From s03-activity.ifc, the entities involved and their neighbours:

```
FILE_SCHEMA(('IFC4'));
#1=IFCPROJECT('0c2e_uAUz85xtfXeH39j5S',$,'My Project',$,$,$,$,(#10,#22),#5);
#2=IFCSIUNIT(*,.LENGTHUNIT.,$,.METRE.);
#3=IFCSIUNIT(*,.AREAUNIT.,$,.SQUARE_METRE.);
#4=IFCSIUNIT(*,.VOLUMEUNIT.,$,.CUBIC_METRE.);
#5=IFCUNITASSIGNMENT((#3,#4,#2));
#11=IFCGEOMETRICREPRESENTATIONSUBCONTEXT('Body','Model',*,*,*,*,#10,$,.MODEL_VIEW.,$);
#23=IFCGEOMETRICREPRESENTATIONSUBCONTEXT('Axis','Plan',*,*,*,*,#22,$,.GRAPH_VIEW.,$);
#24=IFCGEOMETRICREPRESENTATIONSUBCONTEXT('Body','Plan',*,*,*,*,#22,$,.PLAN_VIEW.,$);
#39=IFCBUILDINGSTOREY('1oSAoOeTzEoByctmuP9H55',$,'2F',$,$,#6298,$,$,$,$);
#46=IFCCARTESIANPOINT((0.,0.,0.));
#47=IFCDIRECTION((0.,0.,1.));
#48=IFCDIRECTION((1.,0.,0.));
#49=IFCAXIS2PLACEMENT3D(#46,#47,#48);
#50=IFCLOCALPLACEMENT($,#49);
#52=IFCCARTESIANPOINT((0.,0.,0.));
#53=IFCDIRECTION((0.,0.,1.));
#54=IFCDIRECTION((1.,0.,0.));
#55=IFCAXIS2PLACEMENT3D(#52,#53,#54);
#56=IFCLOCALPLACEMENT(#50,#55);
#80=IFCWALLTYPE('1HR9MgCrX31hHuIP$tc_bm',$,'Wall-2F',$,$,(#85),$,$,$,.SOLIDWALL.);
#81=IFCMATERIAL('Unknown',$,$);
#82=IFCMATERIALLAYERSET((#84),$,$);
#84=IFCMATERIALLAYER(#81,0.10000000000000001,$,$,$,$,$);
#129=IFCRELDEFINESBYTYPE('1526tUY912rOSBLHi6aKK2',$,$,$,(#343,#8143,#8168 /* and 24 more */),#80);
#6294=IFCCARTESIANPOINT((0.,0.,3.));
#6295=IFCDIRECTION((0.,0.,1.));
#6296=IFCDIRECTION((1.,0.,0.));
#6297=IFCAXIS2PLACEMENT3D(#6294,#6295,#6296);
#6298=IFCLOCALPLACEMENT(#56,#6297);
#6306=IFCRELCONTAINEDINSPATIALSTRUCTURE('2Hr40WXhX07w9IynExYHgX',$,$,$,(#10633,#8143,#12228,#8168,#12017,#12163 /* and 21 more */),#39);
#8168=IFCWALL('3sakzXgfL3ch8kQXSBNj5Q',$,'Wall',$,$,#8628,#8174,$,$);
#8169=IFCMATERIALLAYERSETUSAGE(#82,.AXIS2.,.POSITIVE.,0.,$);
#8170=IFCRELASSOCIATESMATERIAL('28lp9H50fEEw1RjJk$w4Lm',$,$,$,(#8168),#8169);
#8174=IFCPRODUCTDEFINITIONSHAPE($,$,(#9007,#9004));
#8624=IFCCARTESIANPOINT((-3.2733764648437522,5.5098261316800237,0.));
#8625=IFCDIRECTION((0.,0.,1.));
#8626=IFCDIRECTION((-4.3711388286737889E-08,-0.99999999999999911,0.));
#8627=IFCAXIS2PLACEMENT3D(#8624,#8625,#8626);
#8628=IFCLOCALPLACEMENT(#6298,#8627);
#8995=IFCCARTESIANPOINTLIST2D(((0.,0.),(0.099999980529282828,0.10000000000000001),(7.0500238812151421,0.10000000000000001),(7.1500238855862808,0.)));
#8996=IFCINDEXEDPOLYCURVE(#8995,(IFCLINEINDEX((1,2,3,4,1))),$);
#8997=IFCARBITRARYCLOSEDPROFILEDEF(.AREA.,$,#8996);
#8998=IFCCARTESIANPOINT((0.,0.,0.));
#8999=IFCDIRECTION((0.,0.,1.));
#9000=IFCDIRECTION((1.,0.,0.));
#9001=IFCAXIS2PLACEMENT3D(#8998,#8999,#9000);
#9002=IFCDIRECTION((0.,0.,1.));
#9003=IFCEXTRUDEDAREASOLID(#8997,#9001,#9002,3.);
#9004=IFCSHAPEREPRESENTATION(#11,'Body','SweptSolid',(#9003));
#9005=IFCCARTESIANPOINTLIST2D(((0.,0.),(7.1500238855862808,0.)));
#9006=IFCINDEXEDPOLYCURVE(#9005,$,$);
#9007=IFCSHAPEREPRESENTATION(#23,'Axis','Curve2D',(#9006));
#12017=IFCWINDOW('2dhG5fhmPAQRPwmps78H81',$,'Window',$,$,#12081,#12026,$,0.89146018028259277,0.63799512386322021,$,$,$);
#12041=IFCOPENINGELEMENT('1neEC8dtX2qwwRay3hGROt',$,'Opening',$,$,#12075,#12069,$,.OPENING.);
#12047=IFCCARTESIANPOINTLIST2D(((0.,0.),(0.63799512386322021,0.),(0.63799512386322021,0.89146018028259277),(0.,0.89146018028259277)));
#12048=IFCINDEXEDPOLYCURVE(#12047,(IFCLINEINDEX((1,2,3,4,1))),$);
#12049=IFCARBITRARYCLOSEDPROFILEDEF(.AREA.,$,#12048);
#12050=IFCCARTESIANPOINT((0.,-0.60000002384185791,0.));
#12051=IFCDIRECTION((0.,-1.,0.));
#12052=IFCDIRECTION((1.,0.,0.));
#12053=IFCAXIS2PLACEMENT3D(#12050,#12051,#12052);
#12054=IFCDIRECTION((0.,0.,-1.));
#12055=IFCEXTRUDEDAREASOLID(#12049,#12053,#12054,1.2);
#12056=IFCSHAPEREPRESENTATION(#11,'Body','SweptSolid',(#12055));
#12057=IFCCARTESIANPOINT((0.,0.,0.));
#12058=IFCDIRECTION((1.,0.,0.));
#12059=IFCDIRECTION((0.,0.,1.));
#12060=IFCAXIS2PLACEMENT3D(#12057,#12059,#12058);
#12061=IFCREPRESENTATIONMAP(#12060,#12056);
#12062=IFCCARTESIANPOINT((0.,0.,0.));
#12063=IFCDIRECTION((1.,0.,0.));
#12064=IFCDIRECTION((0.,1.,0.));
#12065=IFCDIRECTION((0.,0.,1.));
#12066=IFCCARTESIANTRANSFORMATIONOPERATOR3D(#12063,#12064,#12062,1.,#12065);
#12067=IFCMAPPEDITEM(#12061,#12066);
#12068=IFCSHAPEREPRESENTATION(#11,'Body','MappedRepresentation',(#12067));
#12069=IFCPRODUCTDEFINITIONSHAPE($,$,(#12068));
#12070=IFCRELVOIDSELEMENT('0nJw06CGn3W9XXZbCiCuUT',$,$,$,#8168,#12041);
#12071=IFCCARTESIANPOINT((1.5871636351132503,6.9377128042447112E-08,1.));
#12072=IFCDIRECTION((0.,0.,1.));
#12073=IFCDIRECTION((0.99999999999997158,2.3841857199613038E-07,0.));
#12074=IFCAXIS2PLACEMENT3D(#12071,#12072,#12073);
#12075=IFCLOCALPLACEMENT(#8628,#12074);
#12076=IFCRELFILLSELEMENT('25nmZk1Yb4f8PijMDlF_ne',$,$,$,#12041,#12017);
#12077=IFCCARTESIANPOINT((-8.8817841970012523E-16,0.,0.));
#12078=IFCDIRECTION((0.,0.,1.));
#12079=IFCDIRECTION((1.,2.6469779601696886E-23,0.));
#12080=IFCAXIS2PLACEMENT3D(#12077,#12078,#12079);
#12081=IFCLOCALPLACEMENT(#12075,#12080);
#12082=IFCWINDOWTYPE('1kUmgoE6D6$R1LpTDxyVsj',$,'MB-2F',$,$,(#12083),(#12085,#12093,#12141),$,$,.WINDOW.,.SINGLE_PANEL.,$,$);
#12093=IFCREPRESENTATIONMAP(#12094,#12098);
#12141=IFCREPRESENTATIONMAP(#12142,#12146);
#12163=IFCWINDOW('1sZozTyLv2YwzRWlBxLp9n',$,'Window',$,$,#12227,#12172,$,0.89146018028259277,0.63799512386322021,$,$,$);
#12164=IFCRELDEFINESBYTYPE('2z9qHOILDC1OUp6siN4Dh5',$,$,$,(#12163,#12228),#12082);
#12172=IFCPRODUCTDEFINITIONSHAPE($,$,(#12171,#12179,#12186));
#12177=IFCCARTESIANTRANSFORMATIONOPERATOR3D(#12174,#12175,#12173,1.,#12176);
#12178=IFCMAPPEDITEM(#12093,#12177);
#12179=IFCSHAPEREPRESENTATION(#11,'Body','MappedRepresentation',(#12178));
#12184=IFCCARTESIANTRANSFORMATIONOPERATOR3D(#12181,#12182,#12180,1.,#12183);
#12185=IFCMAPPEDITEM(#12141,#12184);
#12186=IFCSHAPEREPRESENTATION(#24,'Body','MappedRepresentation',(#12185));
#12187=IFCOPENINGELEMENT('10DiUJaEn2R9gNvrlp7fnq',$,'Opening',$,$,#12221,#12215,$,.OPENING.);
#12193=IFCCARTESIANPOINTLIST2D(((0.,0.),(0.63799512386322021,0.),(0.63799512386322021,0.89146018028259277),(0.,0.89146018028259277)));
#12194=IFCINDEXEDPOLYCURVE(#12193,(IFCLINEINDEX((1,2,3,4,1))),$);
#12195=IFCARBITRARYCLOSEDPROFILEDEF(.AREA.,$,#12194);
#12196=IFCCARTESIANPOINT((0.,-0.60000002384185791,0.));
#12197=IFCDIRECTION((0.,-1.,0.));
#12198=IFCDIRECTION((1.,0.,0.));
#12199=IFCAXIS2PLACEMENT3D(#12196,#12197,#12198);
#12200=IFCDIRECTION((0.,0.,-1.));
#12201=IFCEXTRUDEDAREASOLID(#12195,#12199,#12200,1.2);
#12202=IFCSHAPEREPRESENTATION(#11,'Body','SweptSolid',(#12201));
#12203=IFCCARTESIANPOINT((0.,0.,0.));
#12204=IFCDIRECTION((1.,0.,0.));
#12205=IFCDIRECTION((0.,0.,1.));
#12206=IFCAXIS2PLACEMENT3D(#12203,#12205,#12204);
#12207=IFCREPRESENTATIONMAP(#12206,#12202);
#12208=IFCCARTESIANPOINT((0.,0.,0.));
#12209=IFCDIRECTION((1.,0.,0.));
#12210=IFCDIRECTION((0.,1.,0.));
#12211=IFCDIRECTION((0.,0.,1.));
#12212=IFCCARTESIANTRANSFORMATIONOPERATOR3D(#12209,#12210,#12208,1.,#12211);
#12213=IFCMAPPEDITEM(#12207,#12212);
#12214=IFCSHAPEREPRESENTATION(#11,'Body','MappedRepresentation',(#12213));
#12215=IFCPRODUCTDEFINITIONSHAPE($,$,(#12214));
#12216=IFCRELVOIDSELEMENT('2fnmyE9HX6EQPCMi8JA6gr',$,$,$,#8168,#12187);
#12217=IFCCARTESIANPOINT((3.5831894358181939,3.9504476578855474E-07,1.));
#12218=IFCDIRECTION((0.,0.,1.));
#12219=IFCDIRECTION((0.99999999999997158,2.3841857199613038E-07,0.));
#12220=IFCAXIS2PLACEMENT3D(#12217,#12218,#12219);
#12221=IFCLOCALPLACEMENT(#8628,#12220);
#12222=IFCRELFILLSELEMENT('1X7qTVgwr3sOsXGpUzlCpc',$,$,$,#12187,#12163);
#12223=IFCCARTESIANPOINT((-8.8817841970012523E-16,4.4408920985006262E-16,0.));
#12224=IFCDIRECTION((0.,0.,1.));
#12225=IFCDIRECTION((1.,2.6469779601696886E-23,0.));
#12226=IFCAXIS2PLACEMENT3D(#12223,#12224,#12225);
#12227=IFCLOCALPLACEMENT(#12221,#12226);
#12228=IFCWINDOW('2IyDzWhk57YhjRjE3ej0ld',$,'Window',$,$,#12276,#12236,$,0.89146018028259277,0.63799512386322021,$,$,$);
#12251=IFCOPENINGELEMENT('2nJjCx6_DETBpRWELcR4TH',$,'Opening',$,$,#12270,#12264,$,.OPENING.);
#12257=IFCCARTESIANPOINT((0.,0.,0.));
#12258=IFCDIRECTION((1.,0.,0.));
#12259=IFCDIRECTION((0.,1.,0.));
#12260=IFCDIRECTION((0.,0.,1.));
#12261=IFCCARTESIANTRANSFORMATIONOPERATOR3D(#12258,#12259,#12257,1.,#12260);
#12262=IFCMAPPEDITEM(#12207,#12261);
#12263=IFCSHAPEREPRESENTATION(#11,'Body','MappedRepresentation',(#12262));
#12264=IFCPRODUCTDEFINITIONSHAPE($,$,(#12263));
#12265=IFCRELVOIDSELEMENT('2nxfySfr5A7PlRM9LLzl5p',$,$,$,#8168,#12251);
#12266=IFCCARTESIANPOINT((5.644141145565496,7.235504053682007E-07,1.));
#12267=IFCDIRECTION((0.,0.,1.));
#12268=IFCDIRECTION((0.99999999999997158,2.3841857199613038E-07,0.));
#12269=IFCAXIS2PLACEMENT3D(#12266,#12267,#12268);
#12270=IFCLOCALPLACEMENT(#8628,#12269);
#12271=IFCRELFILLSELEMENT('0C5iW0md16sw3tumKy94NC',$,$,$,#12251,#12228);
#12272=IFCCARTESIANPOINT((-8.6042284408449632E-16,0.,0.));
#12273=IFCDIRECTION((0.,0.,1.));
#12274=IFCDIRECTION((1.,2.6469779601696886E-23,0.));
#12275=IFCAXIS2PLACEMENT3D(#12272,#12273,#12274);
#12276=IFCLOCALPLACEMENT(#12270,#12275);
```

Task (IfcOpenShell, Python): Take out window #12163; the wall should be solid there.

```python
import ifcopenshell
import ifcopenshell.api.feature
import ifcopenshell.api.root
import ifcopenshell.geom
import ifcopenshell.util.shape

model = ifcopenshell.open("s03-activity.ifc")
settings = ifcopenshell.geom.settings()


def volume(element):
    """Net volume in cubic metres, openings subtracted."""
    shape = ifcopenshell.geom.create_shape(settings, element)
    return ifcopenshell.util.shape.get_volume(shape.geometry)


window = model.by_guid("1sZozTyLv2YwzRWlBxLp9n")
opening = window.FillsVoids[0].RelatingOpeningElement
wall = opening.VoidsElements[0].RelatingBuildingElement
before = volume(wall)

ifcopenshell.api.root.remove_product(model, product=window)
ifcopenshell.api.feature.remove_feature(model, feature=opening)

after = volume(wall)

print(f"wall volume {before:.3f} -> {after:.3f} m3")

model.write("s03-activity_rev.ifc")
```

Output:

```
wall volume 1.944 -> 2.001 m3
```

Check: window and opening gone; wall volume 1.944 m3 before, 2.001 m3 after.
